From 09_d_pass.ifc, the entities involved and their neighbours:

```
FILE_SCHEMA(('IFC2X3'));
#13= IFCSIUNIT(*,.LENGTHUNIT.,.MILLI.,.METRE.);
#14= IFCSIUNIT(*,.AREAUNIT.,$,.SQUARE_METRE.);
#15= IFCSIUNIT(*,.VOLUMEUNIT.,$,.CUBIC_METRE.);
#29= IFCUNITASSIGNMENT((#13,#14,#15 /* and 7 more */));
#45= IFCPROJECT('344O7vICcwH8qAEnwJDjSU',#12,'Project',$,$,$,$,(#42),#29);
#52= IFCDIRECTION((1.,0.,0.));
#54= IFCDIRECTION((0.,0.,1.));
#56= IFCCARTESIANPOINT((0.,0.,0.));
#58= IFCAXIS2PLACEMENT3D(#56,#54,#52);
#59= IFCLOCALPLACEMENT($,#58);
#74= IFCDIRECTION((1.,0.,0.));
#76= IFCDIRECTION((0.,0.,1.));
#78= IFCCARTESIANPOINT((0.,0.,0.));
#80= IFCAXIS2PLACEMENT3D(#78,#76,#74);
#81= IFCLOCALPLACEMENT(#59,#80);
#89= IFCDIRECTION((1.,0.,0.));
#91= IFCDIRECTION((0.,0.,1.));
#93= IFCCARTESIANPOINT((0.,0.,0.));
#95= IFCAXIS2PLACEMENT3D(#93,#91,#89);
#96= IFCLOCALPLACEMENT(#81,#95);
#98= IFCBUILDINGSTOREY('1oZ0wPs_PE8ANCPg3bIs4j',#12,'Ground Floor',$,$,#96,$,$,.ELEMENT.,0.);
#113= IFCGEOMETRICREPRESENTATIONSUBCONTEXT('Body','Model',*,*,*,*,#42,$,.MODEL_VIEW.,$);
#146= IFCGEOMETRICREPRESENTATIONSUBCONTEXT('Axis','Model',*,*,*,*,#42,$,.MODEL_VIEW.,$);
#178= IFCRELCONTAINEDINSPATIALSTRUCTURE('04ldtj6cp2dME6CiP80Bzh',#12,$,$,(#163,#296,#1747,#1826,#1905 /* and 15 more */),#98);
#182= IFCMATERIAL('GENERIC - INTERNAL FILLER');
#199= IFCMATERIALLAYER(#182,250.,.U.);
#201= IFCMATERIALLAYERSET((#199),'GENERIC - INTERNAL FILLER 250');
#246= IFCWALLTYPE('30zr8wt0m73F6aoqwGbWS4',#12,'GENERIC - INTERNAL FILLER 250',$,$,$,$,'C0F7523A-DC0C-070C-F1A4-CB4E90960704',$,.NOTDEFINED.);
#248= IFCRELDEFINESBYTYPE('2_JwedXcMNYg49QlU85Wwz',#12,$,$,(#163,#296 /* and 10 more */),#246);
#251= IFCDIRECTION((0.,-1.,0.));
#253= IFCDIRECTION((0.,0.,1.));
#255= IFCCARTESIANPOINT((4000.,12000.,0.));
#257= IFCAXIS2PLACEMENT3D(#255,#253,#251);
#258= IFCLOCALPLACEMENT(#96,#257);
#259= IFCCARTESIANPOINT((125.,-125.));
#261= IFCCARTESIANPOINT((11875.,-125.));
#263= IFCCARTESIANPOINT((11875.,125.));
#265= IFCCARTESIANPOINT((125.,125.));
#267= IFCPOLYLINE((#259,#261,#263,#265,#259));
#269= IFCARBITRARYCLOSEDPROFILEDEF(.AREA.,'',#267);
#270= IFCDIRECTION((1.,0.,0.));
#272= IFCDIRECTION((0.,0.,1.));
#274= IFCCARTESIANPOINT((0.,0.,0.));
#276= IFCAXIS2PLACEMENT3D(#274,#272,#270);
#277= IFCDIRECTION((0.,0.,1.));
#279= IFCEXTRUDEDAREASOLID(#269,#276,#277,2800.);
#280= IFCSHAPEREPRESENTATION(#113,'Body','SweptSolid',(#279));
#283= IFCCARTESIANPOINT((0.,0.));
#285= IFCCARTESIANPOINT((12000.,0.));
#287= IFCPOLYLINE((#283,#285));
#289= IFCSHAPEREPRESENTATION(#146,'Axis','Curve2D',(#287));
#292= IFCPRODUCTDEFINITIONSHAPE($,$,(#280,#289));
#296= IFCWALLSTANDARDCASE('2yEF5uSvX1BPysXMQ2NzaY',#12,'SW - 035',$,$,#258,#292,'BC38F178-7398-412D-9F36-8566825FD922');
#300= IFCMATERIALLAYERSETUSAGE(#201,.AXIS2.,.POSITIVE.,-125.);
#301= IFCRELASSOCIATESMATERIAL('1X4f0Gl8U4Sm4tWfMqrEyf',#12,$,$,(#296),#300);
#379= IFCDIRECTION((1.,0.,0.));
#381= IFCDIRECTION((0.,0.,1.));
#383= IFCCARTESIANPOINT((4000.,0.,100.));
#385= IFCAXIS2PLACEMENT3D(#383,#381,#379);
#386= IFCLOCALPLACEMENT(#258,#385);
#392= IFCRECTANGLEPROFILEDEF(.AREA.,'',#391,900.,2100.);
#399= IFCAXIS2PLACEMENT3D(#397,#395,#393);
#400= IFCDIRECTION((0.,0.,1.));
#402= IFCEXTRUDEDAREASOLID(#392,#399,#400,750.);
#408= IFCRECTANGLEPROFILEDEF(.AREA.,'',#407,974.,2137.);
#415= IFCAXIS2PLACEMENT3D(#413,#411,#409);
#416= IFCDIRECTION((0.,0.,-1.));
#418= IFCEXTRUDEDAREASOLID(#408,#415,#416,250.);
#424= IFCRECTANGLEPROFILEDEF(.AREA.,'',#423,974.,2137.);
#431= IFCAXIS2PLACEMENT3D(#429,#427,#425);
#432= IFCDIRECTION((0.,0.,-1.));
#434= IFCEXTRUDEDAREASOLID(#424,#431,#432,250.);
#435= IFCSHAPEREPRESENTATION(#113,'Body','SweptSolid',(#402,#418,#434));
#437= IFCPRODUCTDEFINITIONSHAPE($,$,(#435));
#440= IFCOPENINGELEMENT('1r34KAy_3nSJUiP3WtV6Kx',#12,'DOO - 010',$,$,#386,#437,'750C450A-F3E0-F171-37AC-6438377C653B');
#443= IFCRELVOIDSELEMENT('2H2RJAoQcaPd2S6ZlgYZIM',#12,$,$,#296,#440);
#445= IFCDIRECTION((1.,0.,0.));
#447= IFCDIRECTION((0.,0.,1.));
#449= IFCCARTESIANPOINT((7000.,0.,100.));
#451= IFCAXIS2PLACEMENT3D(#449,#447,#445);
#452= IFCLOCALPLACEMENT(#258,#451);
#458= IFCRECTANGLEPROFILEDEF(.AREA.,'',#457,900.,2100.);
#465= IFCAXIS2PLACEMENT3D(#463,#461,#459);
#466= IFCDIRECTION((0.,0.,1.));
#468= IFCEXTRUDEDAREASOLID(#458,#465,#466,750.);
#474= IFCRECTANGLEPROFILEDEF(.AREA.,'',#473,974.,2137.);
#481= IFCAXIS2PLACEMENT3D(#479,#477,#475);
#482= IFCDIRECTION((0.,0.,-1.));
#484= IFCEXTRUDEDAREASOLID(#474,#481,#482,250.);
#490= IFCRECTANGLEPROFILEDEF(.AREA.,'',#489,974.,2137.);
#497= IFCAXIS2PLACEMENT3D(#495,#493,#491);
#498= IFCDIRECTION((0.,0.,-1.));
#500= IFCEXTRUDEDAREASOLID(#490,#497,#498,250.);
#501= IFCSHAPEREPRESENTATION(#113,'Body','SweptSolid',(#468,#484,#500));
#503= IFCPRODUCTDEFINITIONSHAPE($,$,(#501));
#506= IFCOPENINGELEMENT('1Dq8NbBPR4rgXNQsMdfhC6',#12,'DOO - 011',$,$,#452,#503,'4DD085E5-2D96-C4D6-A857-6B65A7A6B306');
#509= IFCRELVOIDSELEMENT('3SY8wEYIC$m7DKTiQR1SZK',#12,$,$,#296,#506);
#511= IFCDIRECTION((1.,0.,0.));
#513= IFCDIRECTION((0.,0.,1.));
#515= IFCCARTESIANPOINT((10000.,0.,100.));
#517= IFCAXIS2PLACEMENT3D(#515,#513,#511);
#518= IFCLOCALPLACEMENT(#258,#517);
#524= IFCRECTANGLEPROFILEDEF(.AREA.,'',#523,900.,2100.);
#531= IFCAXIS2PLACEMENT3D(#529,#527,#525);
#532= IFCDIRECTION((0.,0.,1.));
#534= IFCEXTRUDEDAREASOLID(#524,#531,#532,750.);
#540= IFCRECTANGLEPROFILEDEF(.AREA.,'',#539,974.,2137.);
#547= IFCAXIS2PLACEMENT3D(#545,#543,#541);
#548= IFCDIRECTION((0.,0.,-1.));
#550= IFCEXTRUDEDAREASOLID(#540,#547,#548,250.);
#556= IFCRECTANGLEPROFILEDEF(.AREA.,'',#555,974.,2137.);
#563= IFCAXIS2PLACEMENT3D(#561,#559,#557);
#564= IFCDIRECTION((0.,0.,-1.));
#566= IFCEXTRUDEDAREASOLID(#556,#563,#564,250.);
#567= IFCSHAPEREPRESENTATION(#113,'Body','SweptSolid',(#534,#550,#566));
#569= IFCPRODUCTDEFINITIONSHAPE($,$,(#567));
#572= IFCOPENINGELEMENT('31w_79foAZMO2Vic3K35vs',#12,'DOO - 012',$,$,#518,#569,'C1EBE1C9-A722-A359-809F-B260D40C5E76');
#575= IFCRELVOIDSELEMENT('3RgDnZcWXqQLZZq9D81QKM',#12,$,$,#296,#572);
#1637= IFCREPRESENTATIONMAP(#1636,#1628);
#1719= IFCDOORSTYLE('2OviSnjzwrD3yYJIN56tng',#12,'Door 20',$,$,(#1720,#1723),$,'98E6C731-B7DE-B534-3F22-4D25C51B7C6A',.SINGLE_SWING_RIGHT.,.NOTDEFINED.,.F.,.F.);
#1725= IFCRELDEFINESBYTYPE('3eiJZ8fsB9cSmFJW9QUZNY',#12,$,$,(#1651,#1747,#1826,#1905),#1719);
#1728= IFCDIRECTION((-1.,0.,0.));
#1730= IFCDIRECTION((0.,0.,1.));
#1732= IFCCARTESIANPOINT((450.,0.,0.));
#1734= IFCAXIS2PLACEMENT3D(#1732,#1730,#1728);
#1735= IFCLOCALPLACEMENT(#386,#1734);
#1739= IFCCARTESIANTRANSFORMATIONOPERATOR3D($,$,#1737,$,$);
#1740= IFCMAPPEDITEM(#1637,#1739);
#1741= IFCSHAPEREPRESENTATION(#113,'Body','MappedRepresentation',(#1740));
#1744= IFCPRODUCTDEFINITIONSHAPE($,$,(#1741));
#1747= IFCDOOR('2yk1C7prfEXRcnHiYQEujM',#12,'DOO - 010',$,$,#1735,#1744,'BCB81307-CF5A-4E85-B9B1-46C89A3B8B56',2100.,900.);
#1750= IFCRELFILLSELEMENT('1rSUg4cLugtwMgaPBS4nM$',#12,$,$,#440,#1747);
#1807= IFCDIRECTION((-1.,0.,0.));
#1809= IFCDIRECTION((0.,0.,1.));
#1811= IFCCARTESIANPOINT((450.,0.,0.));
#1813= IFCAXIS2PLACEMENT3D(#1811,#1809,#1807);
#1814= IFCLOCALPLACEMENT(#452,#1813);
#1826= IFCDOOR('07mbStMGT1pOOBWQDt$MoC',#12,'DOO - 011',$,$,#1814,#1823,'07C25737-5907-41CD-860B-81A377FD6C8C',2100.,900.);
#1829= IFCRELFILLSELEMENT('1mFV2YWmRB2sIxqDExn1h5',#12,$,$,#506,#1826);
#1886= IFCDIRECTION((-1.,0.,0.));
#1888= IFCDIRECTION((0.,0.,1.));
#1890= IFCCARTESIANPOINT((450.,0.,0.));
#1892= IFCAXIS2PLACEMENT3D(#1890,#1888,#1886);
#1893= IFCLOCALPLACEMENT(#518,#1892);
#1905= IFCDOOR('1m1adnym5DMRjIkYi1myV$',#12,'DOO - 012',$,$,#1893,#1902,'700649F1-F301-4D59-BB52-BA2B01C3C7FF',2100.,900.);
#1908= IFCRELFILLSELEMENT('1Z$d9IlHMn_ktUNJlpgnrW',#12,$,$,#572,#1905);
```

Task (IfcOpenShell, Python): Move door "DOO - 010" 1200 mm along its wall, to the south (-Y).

```python
import ifcopenshell
import ifcopenshell.api.geometry
import ifcopenshell.util.placement
import ifcopenshell.util.unit

model = ifcopenshell.open("09_d_pass.ifc")
unit_scale = ifcopenshell.util.unit.calculate_unit_scale(model)

door = model.by_guid("2yk1C7prfEXRcnHiYQEujM")
opening = door.FillsVoids[0].RelatingOpeningElement
wall = opening.VoidsElements[0].RelatingBuildingElement

wall_matrix = ifcopenshell.util.placement.get_local_placement(wall.ObjectPlacement)
shift = wall_matrix[:3, 0] * 1.2 / unit_scale
before = ifcopenshell.util.placement.get_local_placement(door.ObjectPlacement)[:3, 3].copy()

# The door is placed relative to its opening, so it follows when the opening moves.
matrix = ifcopenshell.util.placement.get_local_placement(opening.ObjectPlacement)
matrix[:3, 3] += shift
ifcopenshell.api.geometry.edit_object_placement(
    model, product=opening, matrix=matrix, is_si=False, should_transform_children=True
)

after = ifcopenshell.util.placement.get_local_placement(door.ObjectPlacement)[:3, 3]
print("door moved by", (after - before).round(3) + 0.0)

model.write("09_d_pass_v2.ifc")
```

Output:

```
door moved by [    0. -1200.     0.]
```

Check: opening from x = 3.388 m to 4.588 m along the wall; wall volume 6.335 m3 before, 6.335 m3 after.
